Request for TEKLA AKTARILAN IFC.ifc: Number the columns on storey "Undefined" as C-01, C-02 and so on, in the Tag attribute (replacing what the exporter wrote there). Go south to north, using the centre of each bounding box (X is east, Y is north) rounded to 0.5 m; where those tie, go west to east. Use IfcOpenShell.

First a look at what the model holds.

```python
import ifcopenshell
import ifcopenshell.util.element
import ifcopenshell.util.placement

model = ifcopenshell.open("TEKLA AKTARILAN IFC.ifc")
print(model.schema)
storey = next(s for s in model.by_type("IfcBuildingStorey") if s.Name == "Undefined")
columns = [e for e in ifcopenshell.util.element.get_decomposition(storey) if e.is_a("IfcColumn")]
for e in sorted(columns, key=lambda e: e.id()):
    origin = ifcopenshell.util.placement.get_local_placement(e.ObjectPlacement)[:3, 3]
    print(e.id(), e.Tag, e.Name, origin.round(2) + 0.0, sep=" | ")
```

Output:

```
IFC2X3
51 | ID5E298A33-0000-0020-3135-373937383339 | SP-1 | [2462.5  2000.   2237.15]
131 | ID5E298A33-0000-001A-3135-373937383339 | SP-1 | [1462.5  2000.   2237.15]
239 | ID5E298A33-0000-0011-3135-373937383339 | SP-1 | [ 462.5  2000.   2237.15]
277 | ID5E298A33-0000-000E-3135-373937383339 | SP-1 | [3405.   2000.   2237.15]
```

```python
import ifcopenshell
import ifcopenshell.geom
import ifcopenshell.util.element
import ifcopenshell.util.shape

model = ifcopenshell.open("TEKLA AKTARILAN IFC.ifc")
settings = ifcopenshell.geom.settings()
settings.set("use-world-coords", True)


def centre(element):
    shape = ifcopenshell.geom.create_shape(settings, element)
    return ifcopenshell.util.shape.get_bbox_centroid(shape.geometry)


storey = next(s for s in model.by_type("IfcBuildingStorey") if s.Name == "Undefined")
columns = [e for e in ifcopenshell.util.element.get_decomposition(storey) if e.is_a("IfcColumn")]

# Insertion points can sit at a corner or the storey origin, so sort by the geometry (in metres).
centres = {e: centre(e) for e in columns}
columns.sort(key=lambda e: (round(centres[e][1] / 0.5), centres[e][0]))

for i, e in enumerate(columns, start=1):
    number = f"C-{i:02d}"
    e.Tag = number
    print(e.id(), number)

model.write("TEKLA AKTARILAN IFC_edited.ifc")
```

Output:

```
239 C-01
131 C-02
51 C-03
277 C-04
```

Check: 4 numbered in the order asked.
